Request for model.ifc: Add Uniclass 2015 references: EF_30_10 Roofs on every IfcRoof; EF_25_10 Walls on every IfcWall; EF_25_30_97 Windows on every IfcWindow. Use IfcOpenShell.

First a look at what the model holds.

```python
import ifcopenshell

model = ifcopenshell.open("model.ifc")
print(model.schema)
print("classifications:", [c.Name for c in model.by_type("IfcClassification")])
for ifc_class in ("IfcDoor", "IfcRoof", "IfcStair", "IfcWall", "IfcWindow"):
    print(ifc_class, len(model.by_type(ifc_class)))
```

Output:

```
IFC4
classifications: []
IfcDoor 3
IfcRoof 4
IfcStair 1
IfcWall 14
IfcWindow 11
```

```python
import ifcopenshell
import ifcopenshell.api.classification

model = ifcopenshell.open("model.ifc")

system = ifcopenshell.api.classification.add_classification(model, classification="Uniclass 2015")

codes = {
    "IfcRoof": ("EF_30_10", "Roofs"),
    "IfcWall": ("EF_25_10", "Walls"),
    "IfcWindow": ("EF_25_30_97", "Windows"),
}
for ifc_class, (code, name) in codes.items():
    products = model.by_type(ifc_class)
    ifcopenshell.api.classification.add_reference(
        model, products=products, classification=system, identification=code, name=name
    )
    print(code, len(products))

model.write("model_rev.ifc")
```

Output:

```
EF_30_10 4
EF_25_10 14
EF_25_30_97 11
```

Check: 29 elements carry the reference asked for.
